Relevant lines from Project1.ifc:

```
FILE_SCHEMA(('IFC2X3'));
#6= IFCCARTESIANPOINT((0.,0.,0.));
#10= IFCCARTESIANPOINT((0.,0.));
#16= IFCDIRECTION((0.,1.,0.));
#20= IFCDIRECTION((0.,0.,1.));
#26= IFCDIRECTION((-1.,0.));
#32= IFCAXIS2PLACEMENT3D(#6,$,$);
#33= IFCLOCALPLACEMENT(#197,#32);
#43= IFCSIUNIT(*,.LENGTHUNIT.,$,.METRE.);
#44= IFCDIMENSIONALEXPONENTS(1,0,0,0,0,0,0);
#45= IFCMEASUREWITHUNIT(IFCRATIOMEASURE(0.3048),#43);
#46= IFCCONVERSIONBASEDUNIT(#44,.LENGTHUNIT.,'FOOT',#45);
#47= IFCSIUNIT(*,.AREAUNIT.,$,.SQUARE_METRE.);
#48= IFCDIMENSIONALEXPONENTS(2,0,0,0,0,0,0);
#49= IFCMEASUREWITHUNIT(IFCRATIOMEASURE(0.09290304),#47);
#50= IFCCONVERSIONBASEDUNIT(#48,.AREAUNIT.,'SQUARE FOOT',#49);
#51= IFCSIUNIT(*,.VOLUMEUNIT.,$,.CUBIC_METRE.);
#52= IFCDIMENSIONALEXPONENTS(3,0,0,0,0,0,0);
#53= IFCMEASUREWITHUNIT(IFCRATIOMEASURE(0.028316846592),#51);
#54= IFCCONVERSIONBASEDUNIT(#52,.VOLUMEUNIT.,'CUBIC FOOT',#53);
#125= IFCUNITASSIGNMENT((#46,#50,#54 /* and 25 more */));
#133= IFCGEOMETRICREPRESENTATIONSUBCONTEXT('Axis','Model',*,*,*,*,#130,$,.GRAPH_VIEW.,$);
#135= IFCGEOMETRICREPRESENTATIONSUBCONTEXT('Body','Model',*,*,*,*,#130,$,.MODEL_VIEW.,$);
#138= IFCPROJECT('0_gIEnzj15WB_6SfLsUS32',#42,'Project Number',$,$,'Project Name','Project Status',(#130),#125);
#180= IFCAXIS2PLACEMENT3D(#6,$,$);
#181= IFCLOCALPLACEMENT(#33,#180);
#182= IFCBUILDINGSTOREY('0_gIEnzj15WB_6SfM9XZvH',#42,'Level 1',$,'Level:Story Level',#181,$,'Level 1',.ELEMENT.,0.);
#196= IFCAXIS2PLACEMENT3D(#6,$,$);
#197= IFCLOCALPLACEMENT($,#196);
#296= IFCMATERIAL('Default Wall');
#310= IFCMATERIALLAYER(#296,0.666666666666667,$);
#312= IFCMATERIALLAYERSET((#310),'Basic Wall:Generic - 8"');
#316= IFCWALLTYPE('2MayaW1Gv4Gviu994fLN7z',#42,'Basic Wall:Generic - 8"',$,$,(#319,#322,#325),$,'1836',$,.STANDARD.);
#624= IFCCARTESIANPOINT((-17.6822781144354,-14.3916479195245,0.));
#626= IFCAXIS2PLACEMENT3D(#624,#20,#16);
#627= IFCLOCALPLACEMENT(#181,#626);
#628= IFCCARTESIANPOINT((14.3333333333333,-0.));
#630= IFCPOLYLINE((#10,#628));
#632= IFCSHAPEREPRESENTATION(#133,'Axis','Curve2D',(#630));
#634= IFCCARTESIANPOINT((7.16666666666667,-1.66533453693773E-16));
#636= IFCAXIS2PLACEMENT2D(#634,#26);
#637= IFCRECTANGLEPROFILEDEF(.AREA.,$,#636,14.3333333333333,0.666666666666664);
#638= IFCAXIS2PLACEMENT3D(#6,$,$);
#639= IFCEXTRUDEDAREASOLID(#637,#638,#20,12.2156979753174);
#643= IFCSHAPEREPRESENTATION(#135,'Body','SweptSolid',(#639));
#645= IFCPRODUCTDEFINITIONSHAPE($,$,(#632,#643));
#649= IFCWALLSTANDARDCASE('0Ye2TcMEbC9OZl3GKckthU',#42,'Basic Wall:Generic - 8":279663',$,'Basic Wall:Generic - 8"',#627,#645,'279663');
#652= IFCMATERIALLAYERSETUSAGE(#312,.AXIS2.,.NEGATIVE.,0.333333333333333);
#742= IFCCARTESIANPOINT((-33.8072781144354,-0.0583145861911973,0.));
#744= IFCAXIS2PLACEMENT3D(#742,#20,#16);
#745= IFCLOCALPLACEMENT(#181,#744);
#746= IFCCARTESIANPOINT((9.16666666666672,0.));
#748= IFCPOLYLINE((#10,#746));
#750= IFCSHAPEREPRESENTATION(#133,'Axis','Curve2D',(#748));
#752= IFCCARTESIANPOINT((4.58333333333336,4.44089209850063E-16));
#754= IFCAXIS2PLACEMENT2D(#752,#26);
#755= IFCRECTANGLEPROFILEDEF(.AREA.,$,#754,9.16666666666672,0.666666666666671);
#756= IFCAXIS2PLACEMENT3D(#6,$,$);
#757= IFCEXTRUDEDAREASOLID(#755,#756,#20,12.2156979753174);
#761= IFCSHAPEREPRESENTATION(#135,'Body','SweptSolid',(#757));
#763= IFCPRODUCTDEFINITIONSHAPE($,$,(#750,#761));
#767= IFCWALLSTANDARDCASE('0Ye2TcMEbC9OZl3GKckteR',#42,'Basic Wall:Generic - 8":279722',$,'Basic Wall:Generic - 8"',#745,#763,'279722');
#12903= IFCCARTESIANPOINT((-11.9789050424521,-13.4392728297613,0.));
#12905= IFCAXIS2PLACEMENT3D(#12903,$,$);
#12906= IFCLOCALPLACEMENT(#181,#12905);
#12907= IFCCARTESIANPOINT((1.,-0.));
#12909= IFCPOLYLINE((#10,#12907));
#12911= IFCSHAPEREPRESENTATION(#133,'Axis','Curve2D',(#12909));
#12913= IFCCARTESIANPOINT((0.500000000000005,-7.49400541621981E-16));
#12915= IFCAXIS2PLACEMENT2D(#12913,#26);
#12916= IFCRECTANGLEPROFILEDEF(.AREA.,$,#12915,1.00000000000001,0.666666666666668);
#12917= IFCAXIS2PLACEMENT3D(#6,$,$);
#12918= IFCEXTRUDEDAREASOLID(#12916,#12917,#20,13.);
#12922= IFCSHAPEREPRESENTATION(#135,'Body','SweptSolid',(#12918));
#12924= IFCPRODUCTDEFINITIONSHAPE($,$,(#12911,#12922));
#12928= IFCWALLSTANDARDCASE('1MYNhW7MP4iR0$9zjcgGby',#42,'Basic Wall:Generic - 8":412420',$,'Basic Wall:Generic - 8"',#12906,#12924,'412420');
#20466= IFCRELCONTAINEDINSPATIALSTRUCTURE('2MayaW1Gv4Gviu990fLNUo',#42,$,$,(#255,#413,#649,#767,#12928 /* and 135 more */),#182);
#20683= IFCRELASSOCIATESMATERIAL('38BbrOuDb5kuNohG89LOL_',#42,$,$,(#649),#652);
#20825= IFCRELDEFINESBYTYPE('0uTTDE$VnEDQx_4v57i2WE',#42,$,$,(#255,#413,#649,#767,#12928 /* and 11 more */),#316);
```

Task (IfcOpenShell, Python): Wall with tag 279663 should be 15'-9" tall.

```python
import ifcopenshell
import ifcopenshell.geom
import ifcopenshell.util.representation
import ifcopenshell.util.shape
import ifcopenshell.util.unit

model = ifcopenshell.open("Project1.ifc")
unit_scale = ifcopenshell.util.unit.calculate_unit_scale(model)
settings = ifcopenshell.geom.settings()


def volume(element):
    """Net volume in cubic metres, openings subtracted."""
    shape = ifcopenshell.geom.create_shape(settings, element)
    return ifcopenshell.util.shape.get_volume(shape.geometry)


wall = model.by_id(649)
before = volume(wall)

body = ifcopenshell.util.representation.get_representation(wall, "Model", "Body")
solid = body.Items[0]
old_height = solid.Depth
solid.Depth = 189 * 0.0254 / unit_scale
after = volume(wall)

print(f"height {old_height:g} -> {solid.Depth:g}, volume {before:.3f} -> {after:.3f} m3")

model.write("Project1-out.ifc")
```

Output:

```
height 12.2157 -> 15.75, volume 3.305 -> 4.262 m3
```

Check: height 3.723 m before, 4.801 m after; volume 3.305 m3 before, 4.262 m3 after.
